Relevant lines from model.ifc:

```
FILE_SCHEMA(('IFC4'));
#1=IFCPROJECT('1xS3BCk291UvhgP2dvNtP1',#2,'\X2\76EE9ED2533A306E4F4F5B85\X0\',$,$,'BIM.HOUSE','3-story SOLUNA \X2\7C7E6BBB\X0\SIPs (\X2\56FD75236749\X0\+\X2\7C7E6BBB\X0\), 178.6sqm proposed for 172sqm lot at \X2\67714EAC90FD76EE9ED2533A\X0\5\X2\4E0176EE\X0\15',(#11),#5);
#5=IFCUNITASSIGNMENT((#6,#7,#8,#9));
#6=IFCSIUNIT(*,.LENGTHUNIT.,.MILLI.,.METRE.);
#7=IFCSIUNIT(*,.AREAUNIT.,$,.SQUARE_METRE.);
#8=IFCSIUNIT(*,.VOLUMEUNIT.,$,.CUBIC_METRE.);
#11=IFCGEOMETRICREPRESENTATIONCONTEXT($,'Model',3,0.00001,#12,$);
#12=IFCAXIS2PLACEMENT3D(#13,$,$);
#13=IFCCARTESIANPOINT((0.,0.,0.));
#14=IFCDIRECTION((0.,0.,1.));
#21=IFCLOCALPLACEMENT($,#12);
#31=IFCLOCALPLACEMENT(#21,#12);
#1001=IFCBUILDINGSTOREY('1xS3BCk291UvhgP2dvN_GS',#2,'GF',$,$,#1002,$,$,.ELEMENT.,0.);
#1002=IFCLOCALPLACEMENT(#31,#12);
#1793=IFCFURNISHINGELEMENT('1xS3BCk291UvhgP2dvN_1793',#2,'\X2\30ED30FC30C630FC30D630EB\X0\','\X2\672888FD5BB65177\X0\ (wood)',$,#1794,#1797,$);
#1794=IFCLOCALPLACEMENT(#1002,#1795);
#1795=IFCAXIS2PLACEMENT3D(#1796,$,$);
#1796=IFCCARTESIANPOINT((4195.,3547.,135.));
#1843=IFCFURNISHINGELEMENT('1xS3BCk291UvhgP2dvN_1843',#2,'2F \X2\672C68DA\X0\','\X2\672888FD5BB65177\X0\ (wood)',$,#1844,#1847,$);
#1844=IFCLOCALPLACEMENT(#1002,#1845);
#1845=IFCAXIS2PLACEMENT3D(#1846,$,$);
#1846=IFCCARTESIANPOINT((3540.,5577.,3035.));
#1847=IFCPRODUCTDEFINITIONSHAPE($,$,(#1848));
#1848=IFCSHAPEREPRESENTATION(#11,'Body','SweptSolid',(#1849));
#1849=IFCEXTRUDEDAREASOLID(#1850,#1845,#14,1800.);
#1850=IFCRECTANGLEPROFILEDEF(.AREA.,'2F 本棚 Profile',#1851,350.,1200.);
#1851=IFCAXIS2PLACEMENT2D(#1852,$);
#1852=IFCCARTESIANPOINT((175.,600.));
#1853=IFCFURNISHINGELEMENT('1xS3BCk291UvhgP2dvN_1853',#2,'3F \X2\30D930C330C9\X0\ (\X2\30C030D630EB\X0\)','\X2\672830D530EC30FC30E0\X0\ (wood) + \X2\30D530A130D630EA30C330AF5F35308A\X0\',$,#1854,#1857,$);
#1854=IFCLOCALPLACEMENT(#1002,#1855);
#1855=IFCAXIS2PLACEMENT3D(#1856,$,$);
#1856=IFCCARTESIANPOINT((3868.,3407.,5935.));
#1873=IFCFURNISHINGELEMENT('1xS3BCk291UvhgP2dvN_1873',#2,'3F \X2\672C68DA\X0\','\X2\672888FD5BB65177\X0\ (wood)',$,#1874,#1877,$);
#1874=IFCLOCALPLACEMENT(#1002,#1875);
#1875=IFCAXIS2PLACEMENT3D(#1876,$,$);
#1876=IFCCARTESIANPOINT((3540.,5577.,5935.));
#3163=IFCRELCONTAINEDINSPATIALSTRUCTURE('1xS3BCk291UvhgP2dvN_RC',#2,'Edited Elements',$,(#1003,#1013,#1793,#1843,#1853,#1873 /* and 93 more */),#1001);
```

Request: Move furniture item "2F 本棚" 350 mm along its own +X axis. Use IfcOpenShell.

```python
import ifcopenshell
import ifcopenshell.api.geometry
import ifcopenshell.util.placement

model = ifcopenshell.open("model.ifc")

item = model.by_id(1843)
matrix = ifcopenshell.util.placement.get_local_placement(item.ObjectPlacement)
matrix[:3, 3] += matrix[:3, 0] * 350.0
ifcopenshell.api.geometry.edit_object_placement(model, product=item, matrix=matrix, is_si=False)

print(ifcopenshell.util.placement.get_local_placement(item.ObjectPlacement).round(3) + 0.0)

model.write("model_updated.ifc")
```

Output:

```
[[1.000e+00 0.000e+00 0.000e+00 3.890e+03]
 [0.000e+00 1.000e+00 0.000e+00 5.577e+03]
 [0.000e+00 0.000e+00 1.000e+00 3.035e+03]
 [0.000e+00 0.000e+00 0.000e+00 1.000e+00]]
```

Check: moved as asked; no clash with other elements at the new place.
